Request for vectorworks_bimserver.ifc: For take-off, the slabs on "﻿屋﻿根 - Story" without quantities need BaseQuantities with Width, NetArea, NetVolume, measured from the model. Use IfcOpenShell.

First a look at what the model holds.

```python
import ifcopenshell
import ifcopenshell.util.element
import ifcopenshell.util.unit

model = ifcopenshell.open("vectorworks_bimserver.ifc")
print(model.schema)
for unit_type in ("LENGTHUNIT", "AREAUNIT", "VOLUMEUNIT"):
    print(unit_type, ifcopenshell.util.unit.calculate_unit_scale(model, unit_type))
storey = next(s for s in model.by_type("IfcBuildingStorey") if s.Name == '\ufeff屋\ufeff根 - Story')
slabs = [e for e in ifcopenshell.util.element.get_decomposition(storey) if e.is_a("IfcSlab")]
for e in sorted(slabs, key=lambda e: e.id()):
    print(e.id(), e.is_a(), e.Name, list(ifcopenshell.util.element.get_psets(e, qtos_only=True)), sep=" | ")
```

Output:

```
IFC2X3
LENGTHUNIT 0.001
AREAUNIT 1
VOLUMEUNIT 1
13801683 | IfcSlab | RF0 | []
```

```python
import ifcopenshell
import ifcopenshell.api.pset
import ifcopenshell.geom
import ifcopenshell.util.element
import ifcopenshell.util.shape
import ifcopenshell.util.unit

model = ifcopenshell.open("vectorworks_bimserver.ifc")
unit_scale = ifcopenshell.util.unit.calculate_unit_scale(model)
area_scale = ifcopenshell.util.unit.calculate_unit_scale(model, "AREAUNIT")
volume_scale = ifcopenshell.util.unit.calculate_unit_scale(model, "VOLUMEUNIT")
settings = ifcopenshell.geom.settings()

storey = next(s for s in model.by_type("IfcBuildingStorey") if s.Name == '\ufeff屋\ufeff根 - Story')
slabs = [e for e in ifcopenshell.util.element.get_decomposition(storey) if e.is_a("IfcSlab")]

for e in sorted(slabs, key=lambda e: e.id()):
    if ifcopenshell.util.element.get_psets(e, qtos_only=True, should_inherit=False):
        continue
    # Geometry comes back in metres, in the element's own axes.
    shape = ifcopenshell.geom.create_shape(settings, e)
    values = {
        "Width": ifcopenshell.util.shape.get_z(shape.geometry) / unit_scale,
        "NetArea": ifcopenshell.util.shape.get_footprint_area(shape.geometry) / area_scale,
        "NetVolume": ifcopenshell.util.shape.get_volume(shape.geometry) / volume_scale,
    }
    qto = ifcopenshell.api.pset.add_qto(model, product=e, name="BaseQuantities")
    ifcopenshell.api.pset.edit_qto(model, qto=qto, properties=values)
    print(e.id(), {k: round(v, 3) for k, v in values.items()})

model.write("vectorworks_bimserver-out.ifc")
```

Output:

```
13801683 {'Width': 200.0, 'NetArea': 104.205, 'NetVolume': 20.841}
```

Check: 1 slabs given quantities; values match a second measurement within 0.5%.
